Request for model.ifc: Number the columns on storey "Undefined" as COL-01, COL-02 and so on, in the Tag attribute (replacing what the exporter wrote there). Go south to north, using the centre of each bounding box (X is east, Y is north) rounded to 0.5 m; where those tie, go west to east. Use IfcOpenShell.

First a look at what the model holds.

```python
import ifcopenshell
import ifcopenshell.util.element
import ifcopenshell.util.placement

model = ifcopenshell.open("model.ifc")
print(model.schema)
storey = next(s for s in model.by_type("IfcBuildingStorey") if s.Name == "Undefined")
columns = [e for e in ifcopenshell.util.element.get_decomposition(storey) if e.is_a("IfcColumn")]
for e in sorted(columns, key=lambda e: e.id()):
    origin = ifcopenshell.util.placement.get_local_placement(e.ObjectPlacement)[:3, 3]
    print(e.id(), e.Tag, e.Name, origin.round(2) + 0.0, sep=" | ")
```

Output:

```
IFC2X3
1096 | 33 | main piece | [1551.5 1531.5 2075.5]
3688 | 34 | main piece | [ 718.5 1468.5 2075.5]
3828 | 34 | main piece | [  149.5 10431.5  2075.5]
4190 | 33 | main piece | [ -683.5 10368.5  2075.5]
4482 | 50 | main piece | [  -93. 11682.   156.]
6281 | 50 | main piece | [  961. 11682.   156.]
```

```python
import ifcopenshell
import ifcopenshell.geom
import ifcopenshell.util.element
import ifcopenshell.util.shape

model = ifcopenshell.open("model.ifc")
settings = ifcopenshell.geom.settings()
settings.set("use-world-coords", True)


def centre(element):
    shape = ifcopenshell.geom.create_shape(settings, element)
    return ifcopenshell.util.shape.get_bbox_centroid(shape.geometry)


storey = next(s for s in model.by_type("IfcBuildingStorey") if s.Name == "Undefined")
columns = [e for e in ifcopenshell.util.element.get_decomposition(storey) if e.is_a("IfcColumn")]

# Insertion points can sit at a corner or the storey origin, so sort by the geometry (in metres).
centres = {e: centre(e) for e in columns}
columns.sort(key=lambda e: (round(centres[e][1] / 0.5), centres[e][0]))

for i, e in enumerate(columns, start=1):
    number = f"COL-{i:02d}"
    e.Tag = number
    print(e.id(), number)

model.write("model_rev.ifc")
```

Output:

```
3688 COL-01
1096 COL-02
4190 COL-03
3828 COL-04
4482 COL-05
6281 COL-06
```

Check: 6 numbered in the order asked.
